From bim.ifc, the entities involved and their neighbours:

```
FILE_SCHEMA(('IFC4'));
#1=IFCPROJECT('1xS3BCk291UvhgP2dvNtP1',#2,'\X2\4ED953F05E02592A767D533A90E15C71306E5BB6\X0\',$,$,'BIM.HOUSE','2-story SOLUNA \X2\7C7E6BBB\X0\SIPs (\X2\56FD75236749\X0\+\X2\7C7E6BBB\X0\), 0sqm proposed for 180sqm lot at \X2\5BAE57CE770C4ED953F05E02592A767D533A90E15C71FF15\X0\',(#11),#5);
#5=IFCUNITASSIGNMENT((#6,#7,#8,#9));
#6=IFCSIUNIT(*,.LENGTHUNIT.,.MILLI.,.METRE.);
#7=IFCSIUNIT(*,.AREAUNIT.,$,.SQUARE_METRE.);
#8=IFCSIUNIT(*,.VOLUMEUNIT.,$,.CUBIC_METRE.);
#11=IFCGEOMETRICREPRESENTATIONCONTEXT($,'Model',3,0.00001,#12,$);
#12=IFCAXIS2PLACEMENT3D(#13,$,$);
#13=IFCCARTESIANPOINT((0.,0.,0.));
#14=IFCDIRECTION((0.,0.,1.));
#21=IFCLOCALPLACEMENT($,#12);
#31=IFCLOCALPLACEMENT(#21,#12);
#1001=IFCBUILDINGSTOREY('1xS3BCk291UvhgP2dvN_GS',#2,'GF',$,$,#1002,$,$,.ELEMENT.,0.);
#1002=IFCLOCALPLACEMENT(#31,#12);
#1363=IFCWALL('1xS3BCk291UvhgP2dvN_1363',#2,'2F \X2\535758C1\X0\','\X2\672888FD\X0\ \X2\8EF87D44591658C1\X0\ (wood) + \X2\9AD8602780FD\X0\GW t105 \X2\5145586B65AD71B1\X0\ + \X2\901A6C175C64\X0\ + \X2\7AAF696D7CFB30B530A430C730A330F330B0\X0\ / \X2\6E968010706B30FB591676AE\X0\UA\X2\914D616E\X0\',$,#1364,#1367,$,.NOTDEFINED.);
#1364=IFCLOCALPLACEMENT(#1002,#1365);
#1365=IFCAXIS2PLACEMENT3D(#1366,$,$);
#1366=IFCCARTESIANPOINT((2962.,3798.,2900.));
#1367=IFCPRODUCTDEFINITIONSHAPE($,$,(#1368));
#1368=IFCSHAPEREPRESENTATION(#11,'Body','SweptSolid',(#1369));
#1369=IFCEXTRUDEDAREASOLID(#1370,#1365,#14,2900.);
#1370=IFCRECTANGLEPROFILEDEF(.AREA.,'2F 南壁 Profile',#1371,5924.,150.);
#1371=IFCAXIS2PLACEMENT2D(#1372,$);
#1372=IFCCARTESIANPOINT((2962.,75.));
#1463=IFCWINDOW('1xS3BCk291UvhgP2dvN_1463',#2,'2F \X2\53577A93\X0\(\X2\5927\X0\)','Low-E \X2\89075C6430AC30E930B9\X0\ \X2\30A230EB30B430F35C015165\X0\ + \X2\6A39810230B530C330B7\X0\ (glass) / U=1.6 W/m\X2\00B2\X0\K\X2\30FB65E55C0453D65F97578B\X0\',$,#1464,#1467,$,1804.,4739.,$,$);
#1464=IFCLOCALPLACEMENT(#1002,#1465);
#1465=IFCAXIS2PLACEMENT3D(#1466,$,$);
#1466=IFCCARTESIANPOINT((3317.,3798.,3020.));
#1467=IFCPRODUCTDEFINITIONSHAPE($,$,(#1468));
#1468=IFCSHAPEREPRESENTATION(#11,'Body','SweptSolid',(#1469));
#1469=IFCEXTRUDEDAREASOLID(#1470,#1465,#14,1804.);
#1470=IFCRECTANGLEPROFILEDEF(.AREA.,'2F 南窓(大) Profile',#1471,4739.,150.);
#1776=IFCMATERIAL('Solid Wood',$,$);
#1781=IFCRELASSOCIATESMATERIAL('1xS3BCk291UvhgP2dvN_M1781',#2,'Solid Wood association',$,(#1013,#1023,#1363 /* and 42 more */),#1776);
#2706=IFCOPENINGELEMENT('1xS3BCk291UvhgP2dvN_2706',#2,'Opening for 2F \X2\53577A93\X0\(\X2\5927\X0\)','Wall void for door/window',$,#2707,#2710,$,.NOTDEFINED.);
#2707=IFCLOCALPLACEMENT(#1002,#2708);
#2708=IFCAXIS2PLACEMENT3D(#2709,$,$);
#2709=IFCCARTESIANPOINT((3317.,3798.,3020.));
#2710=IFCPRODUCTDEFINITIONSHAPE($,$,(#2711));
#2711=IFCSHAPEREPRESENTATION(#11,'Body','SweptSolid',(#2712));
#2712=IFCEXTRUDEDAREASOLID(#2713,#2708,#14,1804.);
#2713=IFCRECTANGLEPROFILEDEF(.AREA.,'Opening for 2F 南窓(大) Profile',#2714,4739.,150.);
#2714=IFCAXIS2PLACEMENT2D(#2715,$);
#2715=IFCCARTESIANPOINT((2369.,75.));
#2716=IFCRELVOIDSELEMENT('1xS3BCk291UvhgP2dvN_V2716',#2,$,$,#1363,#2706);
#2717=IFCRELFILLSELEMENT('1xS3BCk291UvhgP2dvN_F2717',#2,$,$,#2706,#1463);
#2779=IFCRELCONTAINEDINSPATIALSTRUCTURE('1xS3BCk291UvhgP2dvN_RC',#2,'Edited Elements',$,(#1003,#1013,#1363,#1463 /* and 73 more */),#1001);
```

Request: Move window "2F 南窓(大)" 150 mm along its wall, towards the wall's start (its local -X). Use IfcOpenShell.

```python
import ifcopenshell
import ifcopenshell.api.geometry
import ifcopenshell.util.placement

model = ifcopenshell.open("bim.ifc")

window = model.by_id(1463)
opening = window.FillsVoids[0].RelatingOpeningElement
wall = opening.VoidsElements[0].RelatingBuildingElement

wall_matrix = ifcopenshell.util.placement.get_local_placement(wall.ObjectPlacement)
shift = wall_matrix[:3, 0] * -150.0
before = ifcopenshell.util.placement.get_local_placement(window.ObjectPlacement)[:3, 3].copy()

# The window is not placed relative to its opening, so move both.
for product in (opening, window):
    matrix = ifcopenshell.util.placement.get_local_placement(product.ObjectPlacement)
    matrix[:3, 3] += shift
    ifcopenshell.api.geometry.edit_object_placement(model, product=product, matrix=matrix, is_si=False)

after = ifcopenshell.util.placement.get_local_placement(window.ObjectPlacement)[:3, 3]
print("window moved by", (after - before).round(3) + 0.0)

model.write("bim_v2.ifc")
```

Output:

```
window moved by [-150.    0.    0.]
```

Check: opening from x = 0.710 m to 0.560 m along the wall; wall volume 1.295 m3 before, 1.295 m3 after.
